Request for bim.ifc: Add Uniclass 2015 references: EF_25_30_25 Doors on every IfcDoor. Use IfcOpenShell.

First a look at what the model holds.

```python
import ifcopenshell

model = ifcopenshell.open("bim.ifc")
print(model.schema)
print("classifications:", [c.Name for c in model.by_type("IfcClassification")])
for ifc_class in ("IfcDoor", "IfcRoof", "IfcStair", "IfcWall", "IfcWindow"):
    print(ifc_class, len(model.by_type(ifc_class)))
```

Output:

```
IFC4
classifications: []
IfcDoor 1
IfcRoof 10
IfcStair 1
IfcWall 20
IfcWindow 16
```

```python
import ifcopenshell
import ifcopenshell.api.classification

model = ifcopenshell.open("bim.ifc")

system = ifcopenshell.api.classification.add_classification(model, classification="Uniclass 2015")

codes = {
    "IfcDoor": ("EF_25_30_25", "Doors"),
}
for ifc_class, (code, name) in codes.items():
    products = model.by_type(ifc_class)
    ifcopenshell.api.classification.add_reference(
        model, products=products, classification=system, identification=code, name=name
    )
    print(code, len(products))

model.write("bim_rev.ifc")
```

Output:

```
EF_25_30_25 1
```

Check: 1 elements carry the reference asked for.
